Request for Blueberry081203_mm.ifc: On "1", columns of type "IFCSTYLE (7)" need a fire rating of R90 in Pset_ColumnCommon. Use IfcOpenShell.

First a look at what the model holds.

```python
import ifcopenshell
import ifcopenshell.util.element

model = ifcopenshell.open("Blueberry081203_mm.ifc")
print(model.schema)
storey = next(s for s in model.by_type("IfcBuildingStorey") if s.Name == "1")
columns = [e for e in ifcopenshell.util.element.get_decomposition(storey) if e.is_a("IfcColumn")]
seen = {}
for e in columns:
    element_type = ifcopenshell.util.element.get_type(e)
    key = (element_type.Name if element_type != e and element_type else None, ifcopenshell.util.element.get_pset(e, "Pset_ColumnCommon", "FireRating"))
    seen[key] = seen.get(key, 0) + 1
for (name, value), count in sorted(seen.items(), key=str):
    print(count, "x", name, "|", value)
```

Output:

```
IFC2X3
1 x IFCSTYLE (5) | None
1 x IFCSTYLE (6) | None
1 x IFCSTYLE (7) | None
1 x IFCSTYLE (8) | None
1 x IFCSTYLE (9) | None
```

```python
import ifcopenshell
import ifcopenshell.api.pset
import ifcopenshell.util.element

model = ifcopenshell.open("Blueberry081203_mm.ifc")

storey = next(s for s in model.by_type("IfcBuildingStorey") if s.Name == "1")
columns = [e for e in ifcopenshell.util.element.get_decomposition(storey) if e.is_a("IfcColumn")]

count = 0
for e in columns:
    element_type = ifcopenshell.util.element.get_type(e)
    if element_type in (None, e) or element_type.Name != "IFCSTYLE (7)":
        continue
    # add_pset returns the element's existing set when there is one.
    pset = ifcopenshell.api.pset.add_pset(model, product=e, name="Pset_ColumnCommon")
    ifcopenshell.api.pset.edit_pset(model, pset=pset, properties={"FireRating": "R90"})
    count += 1

print(count, "columns updated")

model.write("Blueberry081203_mm_updated.ifc")
```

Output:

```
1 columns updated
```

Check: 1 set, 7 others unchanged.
